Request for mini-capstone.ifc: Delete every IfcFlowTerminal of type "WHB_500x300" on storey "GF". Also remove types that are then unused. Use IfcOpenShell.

First a look at what the model holds.

```python
import ifcopenshell
import ifcopenshell.util.element

model = ifcopenshell.open("mini-capstone.ifc")
print(model.schema)
storey = next(s for s in model.by_type("IfcBuildingStorey") if s.Name == "GF")
terminals = [e for e in ifcopenshell.util.element.get_decomposition(storey) if e.is_a("IfcFlowTerminal")]
seen = {}
for e in terminals:
    element_type = ifcopenshell.util.element.get_type(e)
    name = element_type.Name if element_type not in (None, e) else None
    seen[name] = seen.get(name, 0) + 1
for name, count in sorted(seen.items(), key=str):
    print(count, "x", name)
```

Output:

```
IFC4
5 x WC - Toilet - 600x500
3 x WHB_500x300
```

```python
import ifcopenshell
import ifcopenshell.api.root
import ifcopenshell.util.element

model = ifcopenshell.open("mini-capstone.ifc")

storey = next(s for s in model.by_type("IfcBuildingStorey") if s.Name == "GF")
terminals = [e for e in ifcopenshell.util.element.get_decomposition(storey) if e.is_a("IfcFlowTerminal")]
targets = [e for e in terminals if (t := ifcopenshell.util.element.get_type(e)) not in (None, e) and t.Name == "WHB_500x300"]
types = {ifcopenshell.util.element.get_type(e) for e in targets} - {None, *targets}

for e in targets:
    ifcopenshell.api.root.remove_product(model, product=e)
print(len(targets), "removed")

unused = [t for t in types if not ifcopenshell.util.element.get_types(t)]
for t in unused:
    ifcopenshell.api.root.remove_product(model, product=t)
print(len(unused), "unused types removed")

model.write("mini-capstone_rev.ifc")
```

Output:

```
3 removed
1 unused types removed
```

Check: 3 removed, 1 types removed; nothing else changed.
